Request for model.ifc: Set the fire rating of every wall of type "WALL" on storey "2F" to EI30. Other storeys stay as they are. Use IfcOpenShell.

First a look at what the model holds.

```python
import ifcopenshell
import ifcopenshell.util.element

model = ifcopenshell.open("model.ifc")
print(model.schema)
storey = next(s for s in model.by_type("IfcBuildingStorey") if s.Name == "2F")
walls = [e for e in ifcopenshell.util.element.get_decomposition(storey) if e.is_a("IfcWall")]
seen = {}
for e in walls:
    element_type = ifcopenshell.util.element.get_type(e)
    key = (element_type.Name if element_type != e and element_type else None, ifcopenshell.util.element.get_pset(e, "Pset_WallCommon", "FireRating"))
    seen[key] = seen.get(key, 0) + 1
for (name, value), count in sorted(seen.items(), key=str):
    print(count, "x", name, "|", value)
```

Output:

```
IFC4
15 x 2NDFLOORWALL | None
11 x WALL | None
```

```python
import ifcopenshell
import ifcopenshell.api.pset
import ifcopenshell.util.element

model = ifcopenshell.open("model.ifc")

storey = next(s for s in model.by_type("IfcBuildingStorey") if s.Name == "2F")
walls = [e for e in ifcopenshell.util.element.get_decomposition(storey) if e.is_a("IfcWall")]

count = 0
for e in walls:
    element_type = ifcopenshell.util.element.get_type(e)
    if element_type in (None, e) or element_type.Name != "WALL":
        continue
    # add_pset returns the element's existing set when there is one.
    pset = ifcopenshell.api.pset.add_pset(model, product=e, name="Pset_WallCommon")
    ifcopenshell.api.pset.edit_pset(model, pset=pset, properties={"FireRating": "EI30"})
    count += 1

print(count, "walls updated")

model.write("model_updated.ifc")
```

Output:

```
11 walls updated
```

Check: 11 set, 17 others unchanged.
